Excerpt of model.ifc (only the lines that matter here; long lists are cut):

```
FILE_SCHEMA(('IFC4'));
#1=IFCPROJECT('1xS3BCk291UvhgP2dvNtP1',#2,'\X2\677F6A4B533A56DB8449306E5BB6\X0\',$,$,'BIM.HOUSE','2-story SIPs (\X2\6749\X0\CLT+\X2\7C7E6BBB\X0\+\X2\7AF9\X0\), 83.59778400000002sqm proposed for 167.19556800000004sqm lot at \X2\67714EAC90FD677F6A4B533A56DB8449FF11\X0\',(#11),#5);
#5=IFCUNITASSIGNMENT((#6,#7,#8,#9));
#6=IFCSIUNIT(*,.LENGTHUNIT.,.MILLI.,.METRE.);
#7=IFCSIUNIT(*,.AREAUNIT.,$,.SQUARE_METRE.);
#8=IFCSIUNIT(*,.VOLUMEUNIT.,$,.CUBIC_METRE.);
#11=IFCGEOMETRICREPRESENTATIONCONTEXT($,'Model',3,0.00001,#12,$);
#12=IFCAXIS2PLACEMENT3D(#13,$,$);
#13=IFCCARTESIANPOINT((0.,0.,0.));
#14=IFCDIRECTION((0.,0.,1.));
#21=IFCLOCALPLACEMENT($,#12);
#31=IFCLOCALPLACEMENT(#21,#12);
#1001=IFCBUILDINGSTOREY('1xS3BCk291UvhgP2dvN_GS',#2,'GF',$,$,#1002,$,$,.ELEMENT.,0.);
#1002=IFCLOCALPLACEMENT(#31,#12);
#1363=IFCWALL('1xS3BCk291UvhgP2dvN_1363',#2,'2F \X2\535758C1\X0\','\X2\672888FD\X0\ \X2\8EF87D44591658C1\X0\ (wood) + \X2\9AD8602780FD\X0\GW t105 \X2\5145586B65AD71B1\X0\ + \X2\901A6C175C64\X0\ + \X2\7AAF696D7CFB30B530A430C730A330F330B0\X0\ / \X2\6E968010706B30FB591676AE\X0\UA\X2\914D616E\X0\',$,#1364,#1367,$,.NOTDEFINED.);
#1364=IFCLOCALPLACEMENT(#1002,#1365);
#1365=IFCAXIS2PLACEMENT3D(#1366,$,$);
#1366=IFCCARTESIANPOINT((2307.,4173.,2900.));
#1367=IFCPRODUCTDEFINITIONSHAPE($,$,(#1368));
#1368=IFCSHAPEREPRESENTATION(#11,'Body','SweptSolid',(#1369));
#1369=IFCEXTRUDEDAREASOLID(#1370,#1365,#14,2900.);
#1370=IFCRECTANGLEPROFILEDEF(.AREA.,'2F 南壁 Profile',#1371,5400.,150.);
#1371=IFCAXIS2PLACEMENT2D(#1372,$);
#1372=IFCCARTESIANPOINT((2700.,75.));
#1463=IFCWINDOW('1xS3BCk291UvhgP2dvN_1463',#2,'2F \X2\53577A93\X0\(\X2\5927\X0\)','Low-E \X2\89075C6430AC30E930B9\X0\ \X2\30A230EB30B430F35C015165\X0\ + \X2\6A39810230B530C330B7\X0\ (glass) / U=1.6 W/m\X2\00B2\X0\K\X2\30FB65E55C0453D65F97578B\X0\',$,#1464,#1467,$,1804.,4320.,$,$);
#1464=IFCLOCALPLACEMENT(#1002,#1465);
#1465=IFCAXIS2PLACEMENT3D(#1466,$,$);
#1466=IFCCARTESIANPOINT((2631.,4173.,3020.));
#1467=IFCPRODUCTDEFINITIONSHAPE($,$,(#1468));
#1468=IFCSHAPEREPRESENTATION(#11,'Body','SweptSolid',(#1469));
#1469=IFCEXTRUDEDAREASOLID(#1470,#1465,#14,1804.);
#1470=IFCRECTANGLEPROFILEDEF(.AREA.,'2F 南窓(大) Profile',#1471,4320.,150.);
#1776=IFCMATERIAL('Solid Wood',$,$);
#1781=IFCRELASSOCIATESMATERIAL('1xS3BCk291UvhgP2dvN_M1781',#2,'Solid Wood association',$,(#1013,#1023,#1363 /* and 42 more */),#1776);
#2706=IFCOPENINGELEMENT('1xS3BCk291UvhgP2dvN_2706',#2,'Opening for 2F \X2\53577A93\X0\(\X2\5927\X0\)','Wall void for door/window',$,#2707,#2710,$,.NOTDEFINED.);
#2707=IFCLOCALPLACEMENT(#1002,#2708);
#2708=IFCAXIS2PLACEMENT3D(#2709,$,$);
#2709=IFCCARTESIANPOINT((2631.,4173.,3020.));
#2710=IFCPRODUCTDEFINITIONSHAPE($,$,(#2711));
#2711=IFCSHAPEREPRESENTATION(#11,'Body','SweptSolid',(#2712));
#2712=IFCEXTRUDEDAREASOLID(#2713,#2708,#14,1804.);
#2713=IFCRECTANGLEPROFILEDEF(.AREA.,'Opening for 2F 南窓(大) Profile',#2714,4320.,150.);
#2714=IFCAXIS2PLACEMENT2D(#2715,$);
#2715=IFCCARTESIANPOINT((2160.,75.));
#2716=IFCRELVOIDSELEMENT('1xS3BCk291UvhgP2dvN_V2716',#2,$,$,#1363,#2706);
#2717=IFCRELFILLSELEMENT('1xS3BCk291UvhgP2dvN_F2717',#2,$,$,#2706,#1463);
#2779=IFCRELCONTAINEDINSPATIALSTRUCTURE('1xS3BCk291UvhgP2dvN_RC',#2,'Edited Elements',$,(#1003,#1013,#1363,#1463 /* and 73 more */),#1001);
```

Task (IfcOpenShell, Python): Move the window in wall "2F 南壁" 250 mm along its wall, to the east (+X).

```python
import ifcopenshell
import ifcopenshell.api.geometry
import ifcopenshell.util.placement
import ifcopenshell.util.unit

model = ifcopenshell.open("model.ifc")
unit_scale = ifcopenshell.util.unit.calculate_unit_scale(model)

window = model.by_guid("1xS3BCk291UvhgP2dvN_1463")
opening = window.FillsVoids[0].RelatingOpeningElement
wall = opening.VoidsElements[0].RelatingBuildingElement

wall_matrix = ifcopenshell.util.placement.get_local_placement(wall.ObjectPlacement)
shift = wall_matrix[:3, 0] * 0.25 / unit_scale
before = ifcopenshell.util.placement.get_local_placement(window.ObjectPlacement)[:3, 3].copy()

# The window is not placed relative to its opening, so move both.
for product in (opening, window):
    matrix = ifcopenshell.util.placement.get_local_placement(product.ObjectPlacement)
    matrix[:3, 3] += shift
    ifcopenshell.api.geometry.edit_object_placement(model, product=product, matrix=matrix, is_si=False)

after = ifcopenshell.util.placement.get_local_placement(window.ObjectPlacement)[:3, 3]
print("window moved by", (after - before).round(3) + 0.0)

model.write("model_updated.ifc")
```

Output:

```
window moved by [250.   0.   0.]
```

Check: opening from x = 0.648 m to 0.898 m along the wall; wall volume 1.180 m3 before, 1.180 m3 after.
